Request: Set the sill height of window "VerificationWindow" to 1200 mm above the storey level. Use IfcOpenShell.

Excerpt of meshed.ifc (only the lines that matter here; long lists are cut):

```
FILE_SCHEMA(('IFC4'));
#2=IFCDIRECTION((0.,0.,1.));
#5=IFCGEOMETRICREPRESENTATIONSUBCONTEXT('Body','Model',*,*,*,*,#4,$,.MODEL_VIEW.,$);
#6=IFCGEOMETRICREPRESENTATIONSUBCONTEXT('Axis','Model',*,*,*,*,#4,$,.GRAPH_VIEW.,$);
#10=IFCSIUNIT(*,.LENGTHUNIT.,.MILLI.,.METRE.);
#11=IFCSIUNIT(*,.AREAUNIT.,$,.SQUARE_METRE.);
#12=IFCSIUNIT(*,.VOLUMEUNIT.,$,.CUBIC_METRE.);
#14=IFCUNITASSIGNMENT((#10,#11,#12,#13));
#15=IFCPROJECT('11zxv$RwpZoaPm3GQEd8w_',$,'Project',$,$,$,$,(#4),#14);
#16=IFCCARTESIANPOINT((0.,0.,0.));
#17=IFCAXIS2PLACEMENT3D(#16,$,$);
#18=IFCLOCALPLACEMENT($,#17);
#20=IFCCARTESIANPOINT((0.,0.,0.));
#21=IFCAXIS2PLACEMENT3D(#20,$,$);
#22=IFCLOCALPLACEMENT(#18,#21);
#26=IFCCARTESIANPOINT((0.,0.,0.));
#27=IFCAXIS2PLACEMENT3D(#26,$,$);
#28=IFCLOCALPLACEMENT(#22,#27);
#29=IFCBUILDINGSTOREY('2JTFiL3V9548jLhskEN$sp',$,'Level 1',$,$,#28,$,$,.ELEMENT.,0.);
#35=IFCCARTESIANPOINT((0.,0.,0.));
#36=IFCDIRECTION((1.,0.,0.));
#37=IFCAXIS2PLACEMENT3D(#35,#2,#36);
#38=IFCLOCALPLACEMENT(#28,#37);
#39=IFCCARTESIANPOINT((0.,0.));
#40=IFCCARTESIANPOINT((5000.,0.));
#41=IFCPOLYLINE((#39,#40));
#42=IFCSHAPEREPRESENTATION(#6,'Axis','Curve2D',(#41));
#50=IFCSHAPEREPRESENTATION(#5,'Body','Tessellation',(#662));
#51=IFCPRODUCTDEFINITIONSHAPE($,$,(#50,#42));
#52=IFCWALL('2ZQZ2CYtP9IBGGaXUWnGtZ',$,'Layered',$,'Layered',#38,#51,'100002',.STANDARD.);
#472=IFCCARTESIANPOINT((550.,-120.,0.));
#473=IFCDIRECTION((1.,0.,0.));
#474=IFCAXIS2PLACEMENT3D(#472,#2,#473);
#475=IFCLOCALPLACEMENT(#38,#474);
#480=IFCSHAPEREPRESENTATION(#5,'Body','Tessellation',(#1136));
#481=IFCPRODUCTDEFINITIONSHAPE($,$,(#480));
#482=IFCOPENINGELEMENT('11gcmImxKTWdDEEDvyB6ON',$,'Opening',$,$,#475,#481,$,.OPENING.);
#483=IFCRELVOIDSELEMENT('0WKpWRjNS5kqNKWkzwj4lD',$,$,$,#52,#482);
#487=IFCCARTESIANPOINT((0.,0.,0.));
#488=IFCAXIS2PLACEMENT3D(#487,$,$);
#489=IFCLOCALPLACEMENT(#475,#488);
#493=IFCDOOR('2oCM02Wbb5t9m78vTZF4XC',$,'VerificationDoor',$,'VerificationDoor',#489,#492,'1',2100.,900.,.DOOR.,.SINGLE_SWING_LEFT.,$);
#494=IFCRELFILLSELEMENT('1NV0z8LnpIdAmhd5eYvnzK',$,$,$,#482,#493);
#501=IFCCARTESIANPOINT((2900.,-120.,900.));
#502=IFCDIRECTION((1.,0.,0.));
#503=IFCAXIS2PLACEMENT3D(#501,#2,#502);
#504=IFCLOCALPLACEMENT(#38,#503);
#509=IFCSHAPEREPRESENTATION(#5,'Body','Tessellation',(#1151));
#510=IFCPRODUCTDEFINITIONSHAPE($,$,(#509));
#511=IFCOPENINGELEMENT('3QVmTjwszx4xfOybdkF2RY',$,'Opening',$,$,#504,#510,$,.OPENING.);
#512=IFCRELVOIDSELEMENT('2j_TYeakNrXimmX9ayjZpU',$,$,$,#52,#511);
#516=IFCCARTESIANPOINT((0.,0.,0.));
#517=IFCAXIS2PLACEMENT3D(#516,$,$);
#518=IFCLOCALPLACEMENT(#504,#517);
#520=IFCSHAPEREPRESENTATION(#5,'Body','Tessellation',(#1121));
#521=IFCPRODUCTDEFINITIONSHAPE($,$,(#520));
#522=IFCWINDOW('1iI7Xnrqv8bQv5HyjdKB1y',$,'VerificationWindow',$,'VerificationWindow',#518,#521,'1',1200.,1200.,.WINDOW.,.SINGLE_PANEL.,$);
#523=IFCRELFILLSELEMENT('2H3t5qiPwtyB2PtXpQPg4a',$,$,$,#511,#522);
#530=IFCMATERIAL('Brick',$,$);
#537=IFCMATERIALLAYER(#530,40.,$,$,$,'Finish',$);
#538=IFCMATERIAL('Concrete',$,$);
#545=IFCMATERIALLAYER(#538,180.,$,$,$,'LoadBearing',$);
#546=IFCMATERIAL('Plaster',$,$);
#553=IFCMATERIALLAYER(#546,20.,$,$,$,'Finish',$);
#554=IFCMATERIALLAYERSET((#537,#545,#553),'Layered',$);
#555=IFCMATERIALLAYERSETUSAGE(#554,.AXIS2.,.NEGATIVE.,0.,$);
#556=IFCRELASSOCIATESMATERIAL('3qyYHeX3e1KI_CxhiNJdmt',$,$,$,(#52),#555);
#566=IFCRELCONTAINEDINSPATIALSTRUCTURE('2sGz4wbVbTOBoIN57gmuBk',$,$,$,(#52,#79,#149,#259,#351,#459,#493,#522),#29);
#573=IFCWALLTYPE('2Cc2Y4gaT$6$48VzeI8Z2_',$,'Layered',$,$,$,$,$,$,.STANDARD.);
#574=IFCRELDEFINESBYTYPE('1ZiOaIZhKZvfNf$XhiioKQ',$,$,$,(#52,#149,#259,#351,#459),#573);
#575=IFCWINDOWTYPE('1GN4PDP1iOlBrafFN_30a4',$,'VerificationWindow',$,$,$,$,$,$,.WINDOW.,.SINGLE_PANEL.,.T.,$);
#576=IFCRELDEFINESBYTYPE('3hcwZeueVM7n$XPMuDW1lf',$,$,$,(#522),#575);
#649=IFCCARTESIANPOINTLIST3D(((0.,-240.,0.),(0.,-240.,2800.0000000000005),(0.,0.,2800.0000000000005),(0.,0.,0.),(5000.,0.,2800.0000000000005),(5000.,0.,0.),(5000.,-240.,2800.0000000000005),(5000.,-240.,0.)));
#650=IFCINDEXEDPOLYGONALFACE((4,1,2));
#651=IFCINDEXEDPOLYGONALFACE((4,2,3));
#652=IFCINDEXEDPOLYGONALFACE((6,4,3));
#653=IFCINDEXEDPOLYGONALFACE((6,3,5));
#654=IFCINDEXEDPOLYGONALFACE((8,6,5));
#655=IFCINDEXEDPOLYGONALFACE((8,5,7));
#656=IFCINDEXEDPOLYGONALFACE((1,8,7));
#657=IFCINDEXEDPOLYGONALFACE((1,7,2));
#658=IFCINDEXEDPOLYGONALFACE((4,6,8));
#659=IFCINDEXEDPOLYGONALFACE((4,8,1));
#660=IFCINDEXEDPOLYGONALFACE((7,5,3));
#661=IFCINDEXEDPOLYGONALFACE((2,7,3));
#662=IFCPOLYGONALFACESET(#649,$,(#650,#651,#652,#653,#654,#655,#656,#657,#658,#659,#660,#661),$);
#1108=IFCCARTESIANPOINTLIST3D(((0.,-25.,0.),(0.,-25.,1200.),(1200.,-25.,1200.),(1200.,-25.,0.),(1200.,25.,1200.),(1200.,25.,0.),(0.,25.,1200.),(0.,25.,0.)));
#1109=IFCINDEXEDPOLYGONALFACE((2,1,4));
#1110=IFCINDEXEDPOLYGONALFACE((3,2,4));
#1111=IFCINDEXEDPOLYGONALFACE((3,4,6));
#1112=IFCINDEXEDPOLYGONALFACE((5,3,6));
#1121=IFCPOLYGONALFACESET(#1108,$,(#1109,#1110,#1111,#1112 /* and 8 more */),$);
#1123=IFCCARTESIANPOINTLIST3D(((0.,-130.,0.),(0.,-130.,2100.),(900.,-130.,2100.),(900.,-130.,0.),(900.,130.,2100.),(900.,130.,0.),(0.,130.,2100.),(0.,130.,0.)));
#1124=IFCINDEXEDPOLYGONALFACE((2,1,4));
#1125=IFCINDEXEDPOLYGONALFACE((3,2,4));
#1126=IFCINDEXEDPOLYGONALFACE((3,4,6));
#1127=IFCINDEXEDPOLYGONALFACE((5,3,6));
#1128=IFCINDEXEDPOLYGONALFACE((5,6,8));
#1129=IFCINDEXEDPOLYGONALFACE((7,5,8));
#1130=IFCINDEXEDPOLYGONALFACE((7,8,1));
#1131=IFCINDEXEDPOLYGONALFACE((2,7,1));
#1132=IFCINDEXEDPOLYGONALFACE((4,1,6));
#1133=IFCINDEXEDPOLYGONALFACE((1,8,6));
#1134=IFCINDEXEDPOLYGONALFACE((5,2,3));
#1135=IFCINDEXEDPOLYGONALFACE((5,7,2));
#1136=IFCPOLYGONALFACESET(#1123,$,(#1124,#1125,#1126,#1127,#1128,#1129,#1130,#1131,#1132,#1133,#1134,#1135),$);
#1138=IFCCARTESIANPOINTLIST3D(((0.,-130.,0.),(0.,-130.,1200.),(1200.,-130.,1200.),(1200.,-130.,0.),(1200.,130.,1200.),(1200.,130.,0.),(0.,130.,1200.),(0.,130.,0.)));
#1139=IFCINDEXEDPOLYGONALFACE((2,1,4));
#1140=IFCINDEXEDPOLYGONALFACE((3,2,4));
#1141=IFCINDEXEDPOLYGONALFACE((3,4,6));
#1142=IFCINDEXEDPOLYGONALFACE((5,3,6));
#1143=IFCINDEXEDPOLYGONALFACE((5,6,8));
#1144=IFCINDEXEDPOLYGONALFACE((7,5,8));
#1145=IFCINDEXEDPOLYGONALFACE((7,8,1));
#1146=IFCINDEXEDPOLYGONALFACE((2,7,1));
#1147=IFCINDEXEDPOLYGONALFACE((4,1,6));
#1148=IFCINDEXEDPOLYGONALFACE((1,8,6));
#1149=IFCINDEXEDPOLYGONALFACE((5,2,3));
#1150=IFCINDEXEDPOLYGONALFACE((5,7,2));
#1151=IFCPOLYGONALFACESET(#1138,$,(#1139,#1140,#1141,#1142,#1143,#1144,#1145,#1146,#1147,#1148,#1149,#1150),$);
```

```python
import numpy as np
import ifcopenshell
import ifcopenshell.api.geometry
import ifcopenshell.geom
import ifcopenshell.util.element
import ifcopenshell.util.placement
import ifcopenshell.util.shape
import ifcopenshell.util.unit

model = ifcopenshell.open("meshed.ifc")
unit_scale = ifcopenshell.util.unit.calculate_unit_scale(model)

window = model.by_guid("1iI7Xnrqv8bQv5HyjdKB1y")
opening = window.FillsVoids[0].RelatingOpeningElement
storey = ifcopenshell.util.element.get_container(window, ifc_class="IfcBuildingStorey")
level = ifcopenshell.util.placement.get_local_placement(storey.ObjectPlacement)[2, 3]

# The opening's origin need not be at the sill, so measure its lowest point.
shape = ifcopenshell.geom.create_shape(ifcopenshell.geom.settings(), opening)
bottom = ifcopenshell.util.shape.get_shape_bottom_elevation(shape, shape.geometry) / unit_scale
dz = level + 1200.0 - bottom

shift = np.array([0.0, 0.0, dz])
# The window is placed relative to its opening, so it follows when the opening moves.
matrix = ifcopenshell.util.placement.get_local_placement(opening.ObjectPlacement)
matrix[:3, 3] += shift
ifcopenshell.api.geometry.edit_object_placement(
    model, product=opening, matrix=matrix, is_si=False, should_transform_children=True
)

print(f"moved by {dz * unit_scale:+.3f} m")

model.write("meshed_v2.ifc")
```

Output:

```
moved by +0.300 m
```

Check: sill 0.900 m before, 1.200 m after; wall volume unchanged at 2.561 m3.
